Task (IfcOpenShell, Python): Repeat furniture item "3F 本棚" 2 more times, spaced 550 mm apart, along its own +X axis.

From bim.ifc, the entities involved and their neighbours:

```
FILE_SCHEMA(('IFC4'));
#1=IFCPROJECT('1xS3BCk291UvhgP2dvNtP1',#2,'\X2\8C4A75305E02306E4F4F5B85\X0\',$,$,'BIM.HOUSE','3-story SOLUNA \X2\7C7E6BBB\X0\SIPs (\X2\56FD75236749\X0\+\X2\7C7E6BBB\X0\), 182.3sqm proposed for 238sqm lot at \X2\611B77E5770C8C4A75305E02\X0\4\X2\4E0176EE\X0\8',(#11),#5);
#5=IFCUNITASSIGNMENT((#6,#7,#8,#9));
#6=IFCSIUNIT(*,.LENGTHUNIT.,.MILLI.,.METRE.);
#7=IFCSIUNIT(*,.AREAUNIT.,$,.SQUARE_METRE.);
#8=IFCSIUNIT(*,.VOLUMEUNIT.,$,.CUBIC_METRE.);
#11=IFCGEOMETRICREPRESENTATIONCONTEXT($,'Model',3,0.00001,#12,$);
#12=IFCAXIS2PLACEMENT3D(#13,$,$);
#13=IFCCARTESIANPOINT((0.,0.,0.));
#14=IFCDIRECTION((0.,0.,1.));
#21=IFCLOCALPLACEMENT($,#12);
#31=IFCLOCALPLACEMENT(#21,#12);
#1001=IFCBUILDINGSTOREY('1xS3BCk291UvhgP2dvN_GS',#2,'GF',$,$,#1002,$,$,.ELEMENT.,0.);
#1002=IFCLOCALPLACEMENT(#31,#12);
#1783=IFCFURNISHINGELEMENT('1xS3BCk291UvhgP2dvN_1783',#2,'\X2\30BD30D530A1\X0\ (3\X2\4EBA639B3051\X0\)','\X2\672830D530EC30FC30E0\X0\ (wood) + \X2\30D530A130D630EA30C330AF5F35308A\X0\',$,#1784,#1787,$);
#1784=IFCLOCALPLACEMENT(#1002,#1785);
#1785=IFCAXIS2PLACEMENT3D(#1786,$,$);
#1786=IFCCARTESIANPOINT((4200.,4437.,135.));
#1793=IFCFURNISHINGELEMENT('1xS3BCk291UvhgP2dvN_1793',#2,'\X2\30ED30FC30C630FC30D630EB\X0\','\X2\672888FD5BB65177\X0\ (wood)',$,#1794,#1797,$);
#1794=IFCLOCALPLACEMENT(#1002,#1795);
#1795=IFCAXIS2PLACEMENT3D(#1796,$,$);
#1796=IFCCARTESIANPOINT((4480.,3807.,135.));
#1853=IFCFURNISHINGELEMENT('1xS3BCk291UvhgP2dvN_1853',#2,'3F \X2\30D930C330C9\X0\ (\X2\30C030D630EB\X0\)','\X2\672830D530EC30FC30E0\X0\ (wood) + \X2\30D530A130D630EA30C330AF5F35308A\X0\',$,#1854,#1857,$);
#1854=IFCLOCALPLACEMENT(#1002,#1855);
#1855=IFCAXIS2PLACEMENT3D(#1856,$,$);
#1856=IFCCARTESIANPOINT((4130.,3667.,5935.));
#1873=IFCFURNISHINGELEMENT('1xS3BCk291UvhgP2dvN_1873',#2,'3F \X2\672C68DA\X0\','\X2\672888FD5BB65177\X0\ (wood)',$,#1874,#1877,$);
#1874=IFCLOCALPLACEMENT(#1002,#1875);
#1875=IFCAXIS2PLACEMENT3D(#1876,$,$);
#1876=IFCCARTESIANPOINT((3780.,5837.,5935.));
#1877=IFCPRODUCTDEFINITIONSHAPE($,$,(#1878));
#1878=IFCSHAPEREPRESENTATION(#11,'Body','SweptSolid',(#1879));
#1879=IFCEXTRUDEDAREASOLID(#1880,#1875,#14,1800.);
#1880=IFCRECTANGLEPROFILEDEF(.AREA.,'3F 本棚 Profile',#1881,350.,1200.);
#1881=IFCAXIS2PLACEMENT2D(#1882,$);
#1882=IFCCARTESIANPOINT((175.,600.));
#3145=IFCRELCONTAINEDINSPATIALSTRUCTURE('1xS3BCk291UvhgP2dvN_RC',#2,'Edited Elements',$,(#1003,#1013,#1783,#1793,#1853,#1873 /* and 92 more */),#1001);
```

```python
import ifcopenshell
import ifcopenshell.api.geometry
import ifcopenshell.api.root
import ifcopenshell.util.element
import ifcopenshell.util.placement
import ifcopenshell.util.unit

model = ifcopenshell.open("bim.ifc")
unit_scale = ifcopenshell.util.unit.calculate_unit_scale(model)


def reuse_history(source, copy):
    """copy_class also copies each property set's owner history, people and application; keep the originals."""
    for rel in copy.IsDefinedBy:
        if rel.is_a("IfcRelDefinesByProperties") and (history := rel.RelatingPropertyDefinition.OwnerHistory):
            rel.RelatingPropertyDefinition.OwnerHistory = source.OwnerHistory
            ifcopenshell.util.element.remove_deep2(model, history)


source = model.by_guid("1xS3BCk291UvhgP2dvN_1873")
base = ifcopenshell.util.placement.get_local_placement(source.ObjectPlacement)
step = base[:3, 0] * 0.55 / unit_scale

for i in range(1, 3):
    copy = ifcopenshell.api.root.copy_class(model, product=source)
    copy.Representation = ifcopenshell.util.element.copy_deep(
        model, source.Representation, exclude=["IfcGeometricRepresentationContext", "IfcRepresentationMap"]
    )
    reuse_history(source, copy)
    matrix = base.copy()
    matrix[:3, 3] += i * step
    print("added at", matrix[:3, 3].round(3) + 0.0)
    ifcopenshell.api.geometry.edit_object_placement(model, product=copy, matrix=matrix, is_si=False)

model.write("bim-out.ifc")
```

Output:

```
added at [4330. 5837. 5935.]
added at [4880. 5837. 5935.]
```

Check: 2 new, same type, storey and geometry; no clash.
